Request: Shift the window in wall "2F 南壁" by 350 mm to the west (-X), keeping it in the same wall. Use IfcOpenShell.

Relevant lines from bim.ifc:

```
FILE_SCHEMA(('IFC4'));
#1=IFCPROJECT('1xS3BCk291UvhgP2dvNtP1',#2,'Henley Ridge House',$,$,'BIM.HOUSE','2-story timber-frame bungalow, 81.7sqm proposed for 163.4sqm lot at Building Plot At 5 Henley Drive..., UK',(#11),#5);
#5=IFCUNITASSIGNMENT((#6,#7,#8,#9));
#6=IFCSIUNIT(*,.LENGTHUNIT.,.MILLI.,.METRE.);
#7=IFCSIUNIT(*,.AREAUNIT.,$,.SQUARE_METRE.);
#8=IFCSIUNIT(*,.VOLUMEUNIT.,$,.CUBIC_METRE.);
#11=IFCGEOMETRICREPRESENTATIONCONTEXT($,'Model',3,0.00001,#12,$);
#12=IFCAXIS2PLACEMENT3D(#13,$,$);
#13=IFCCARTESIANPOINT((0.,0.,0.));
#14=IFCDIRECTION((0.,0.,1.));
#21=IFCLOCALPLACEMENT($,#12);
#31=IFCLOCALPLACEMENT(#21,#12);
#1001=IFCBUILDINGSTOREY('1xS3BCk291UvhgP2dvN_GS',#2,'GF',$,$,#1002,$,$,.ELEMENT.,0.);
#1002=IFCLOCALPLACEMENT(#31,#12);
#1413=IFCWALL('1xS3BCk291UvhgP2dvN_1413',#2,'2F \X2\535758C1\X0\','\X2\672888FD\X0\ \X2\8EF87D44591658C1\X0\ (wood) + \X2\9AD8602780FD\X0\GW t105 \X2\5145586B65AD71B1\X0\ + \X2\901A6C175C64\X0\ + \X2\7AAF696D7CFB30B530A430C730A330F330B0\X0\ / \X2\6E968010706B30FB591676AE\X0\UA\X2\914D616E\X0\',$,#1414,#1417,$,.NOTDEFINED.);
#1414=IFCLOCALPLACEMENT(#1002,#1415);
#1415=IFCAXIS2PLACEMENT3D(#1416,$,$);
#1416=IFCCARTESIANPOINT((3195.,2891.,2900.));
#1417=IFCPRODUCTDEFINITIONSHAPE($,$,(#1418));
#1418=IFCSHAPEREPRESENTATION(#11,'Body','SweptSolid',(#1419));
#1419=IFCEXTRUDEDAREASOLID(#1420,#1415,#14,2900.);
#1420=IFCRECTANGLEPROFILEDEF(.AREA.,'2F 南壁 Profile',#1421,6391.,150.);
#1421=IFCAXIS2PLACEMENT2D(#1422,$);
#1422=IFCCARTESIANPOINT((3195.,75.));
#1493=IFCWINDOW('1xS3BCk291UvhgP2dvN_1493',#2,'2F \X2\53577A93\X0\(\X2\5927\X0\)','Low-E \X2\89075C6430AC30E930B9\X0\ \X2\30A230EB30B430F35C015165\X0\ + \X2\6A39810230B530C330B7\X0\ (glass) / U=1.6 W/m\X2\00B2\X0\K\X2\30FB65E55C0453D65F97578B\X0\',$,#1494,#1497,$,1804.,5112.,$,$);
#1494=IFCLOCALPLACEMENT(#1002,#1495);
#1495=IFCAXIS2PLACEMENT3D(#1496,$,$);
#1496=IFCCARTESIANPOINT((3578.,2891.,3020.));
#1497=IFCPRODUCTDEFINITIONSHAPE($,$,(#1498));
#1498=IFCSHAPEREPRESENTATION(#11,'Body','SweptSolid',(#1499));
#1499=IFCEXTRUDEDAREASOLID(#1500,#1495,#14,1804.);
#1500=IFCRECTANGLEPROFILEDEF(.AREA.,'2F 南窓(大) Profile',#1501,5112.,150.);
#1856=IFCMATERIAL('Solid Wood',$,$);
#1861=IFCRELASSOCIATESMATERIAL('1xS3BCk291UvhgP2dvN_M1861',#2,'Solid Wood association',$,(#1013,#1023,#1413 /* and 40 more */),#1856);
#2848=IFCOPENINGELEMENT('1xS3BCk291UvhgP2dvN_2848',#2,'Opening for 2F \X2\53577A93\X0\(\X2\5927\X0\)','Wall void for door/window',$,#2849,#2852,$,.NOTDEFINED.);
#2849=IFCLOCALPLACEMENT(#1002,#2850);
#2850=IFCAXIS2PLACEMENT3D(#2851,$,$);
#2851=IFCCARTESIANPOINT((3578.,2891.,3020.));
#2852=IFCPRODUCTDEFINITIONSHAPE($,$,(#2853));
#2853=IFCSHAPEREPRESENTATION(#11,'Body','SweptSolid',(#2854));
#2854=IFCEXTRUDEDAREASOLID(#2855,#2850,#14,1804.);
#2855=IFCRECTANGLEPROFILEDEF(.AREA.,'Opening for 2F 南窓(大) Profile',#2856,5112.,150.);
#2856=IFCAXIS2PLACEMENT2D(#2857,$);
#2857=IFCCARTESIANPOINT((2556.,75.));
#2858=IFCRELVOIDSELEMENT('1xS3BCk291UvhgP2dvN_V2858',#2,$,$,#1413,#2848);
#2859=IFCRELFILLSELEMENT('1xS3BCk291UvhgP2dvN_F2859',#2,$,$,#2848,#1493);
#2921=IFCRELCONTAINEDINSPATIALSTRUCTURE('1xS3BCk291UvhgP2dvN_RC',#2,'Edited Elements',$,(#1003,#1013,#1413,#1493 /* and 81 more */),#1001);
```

```python
import ifcopenshell
import ifcopenshell.api.geometry
import ifcopenshell.util.placement

model = ifcopenshell.open("bim.ifc")

window = model.by_guid("1xS3BCk291UvhgP2dvN_1493")
opening = window.FillsVoids[0].RelatingOpeningElement
wall = opening.VoidsElements[0].RelatingBuildingElement

wall_matrix = ifcopenshell.util.placement.get_local_placement(wall.ObjectPlacement)
shift = wall_matrix[:3, 0] * -350.0
before = ifcopenshell.util.placement.get_local_placement(window.ObjectPlacement)[:3, 3].copy()

# The window is not placed relative to its opening, so move both.
for product in (opening, window):
    matrix = ifcopenshell.util.placement.get_local_placement(product.ObjectPlacement)
    matrix[:3, 3] += shift
    ifcopenshell.api.geometry.edit_object_placement(model, product=product, matrix=matrix, is_si=False)

after = ifcopenshell.util.placement.get_local_placement(window.ObjectPlacement)[:3, 3]
print("window moved by", (after - before).round(3) + 0.0)

model.write("bim_updated.ifc")
```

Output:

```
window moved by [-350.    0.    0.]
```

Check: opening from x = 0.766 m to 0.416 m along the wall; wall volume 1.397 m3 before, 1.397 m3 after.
